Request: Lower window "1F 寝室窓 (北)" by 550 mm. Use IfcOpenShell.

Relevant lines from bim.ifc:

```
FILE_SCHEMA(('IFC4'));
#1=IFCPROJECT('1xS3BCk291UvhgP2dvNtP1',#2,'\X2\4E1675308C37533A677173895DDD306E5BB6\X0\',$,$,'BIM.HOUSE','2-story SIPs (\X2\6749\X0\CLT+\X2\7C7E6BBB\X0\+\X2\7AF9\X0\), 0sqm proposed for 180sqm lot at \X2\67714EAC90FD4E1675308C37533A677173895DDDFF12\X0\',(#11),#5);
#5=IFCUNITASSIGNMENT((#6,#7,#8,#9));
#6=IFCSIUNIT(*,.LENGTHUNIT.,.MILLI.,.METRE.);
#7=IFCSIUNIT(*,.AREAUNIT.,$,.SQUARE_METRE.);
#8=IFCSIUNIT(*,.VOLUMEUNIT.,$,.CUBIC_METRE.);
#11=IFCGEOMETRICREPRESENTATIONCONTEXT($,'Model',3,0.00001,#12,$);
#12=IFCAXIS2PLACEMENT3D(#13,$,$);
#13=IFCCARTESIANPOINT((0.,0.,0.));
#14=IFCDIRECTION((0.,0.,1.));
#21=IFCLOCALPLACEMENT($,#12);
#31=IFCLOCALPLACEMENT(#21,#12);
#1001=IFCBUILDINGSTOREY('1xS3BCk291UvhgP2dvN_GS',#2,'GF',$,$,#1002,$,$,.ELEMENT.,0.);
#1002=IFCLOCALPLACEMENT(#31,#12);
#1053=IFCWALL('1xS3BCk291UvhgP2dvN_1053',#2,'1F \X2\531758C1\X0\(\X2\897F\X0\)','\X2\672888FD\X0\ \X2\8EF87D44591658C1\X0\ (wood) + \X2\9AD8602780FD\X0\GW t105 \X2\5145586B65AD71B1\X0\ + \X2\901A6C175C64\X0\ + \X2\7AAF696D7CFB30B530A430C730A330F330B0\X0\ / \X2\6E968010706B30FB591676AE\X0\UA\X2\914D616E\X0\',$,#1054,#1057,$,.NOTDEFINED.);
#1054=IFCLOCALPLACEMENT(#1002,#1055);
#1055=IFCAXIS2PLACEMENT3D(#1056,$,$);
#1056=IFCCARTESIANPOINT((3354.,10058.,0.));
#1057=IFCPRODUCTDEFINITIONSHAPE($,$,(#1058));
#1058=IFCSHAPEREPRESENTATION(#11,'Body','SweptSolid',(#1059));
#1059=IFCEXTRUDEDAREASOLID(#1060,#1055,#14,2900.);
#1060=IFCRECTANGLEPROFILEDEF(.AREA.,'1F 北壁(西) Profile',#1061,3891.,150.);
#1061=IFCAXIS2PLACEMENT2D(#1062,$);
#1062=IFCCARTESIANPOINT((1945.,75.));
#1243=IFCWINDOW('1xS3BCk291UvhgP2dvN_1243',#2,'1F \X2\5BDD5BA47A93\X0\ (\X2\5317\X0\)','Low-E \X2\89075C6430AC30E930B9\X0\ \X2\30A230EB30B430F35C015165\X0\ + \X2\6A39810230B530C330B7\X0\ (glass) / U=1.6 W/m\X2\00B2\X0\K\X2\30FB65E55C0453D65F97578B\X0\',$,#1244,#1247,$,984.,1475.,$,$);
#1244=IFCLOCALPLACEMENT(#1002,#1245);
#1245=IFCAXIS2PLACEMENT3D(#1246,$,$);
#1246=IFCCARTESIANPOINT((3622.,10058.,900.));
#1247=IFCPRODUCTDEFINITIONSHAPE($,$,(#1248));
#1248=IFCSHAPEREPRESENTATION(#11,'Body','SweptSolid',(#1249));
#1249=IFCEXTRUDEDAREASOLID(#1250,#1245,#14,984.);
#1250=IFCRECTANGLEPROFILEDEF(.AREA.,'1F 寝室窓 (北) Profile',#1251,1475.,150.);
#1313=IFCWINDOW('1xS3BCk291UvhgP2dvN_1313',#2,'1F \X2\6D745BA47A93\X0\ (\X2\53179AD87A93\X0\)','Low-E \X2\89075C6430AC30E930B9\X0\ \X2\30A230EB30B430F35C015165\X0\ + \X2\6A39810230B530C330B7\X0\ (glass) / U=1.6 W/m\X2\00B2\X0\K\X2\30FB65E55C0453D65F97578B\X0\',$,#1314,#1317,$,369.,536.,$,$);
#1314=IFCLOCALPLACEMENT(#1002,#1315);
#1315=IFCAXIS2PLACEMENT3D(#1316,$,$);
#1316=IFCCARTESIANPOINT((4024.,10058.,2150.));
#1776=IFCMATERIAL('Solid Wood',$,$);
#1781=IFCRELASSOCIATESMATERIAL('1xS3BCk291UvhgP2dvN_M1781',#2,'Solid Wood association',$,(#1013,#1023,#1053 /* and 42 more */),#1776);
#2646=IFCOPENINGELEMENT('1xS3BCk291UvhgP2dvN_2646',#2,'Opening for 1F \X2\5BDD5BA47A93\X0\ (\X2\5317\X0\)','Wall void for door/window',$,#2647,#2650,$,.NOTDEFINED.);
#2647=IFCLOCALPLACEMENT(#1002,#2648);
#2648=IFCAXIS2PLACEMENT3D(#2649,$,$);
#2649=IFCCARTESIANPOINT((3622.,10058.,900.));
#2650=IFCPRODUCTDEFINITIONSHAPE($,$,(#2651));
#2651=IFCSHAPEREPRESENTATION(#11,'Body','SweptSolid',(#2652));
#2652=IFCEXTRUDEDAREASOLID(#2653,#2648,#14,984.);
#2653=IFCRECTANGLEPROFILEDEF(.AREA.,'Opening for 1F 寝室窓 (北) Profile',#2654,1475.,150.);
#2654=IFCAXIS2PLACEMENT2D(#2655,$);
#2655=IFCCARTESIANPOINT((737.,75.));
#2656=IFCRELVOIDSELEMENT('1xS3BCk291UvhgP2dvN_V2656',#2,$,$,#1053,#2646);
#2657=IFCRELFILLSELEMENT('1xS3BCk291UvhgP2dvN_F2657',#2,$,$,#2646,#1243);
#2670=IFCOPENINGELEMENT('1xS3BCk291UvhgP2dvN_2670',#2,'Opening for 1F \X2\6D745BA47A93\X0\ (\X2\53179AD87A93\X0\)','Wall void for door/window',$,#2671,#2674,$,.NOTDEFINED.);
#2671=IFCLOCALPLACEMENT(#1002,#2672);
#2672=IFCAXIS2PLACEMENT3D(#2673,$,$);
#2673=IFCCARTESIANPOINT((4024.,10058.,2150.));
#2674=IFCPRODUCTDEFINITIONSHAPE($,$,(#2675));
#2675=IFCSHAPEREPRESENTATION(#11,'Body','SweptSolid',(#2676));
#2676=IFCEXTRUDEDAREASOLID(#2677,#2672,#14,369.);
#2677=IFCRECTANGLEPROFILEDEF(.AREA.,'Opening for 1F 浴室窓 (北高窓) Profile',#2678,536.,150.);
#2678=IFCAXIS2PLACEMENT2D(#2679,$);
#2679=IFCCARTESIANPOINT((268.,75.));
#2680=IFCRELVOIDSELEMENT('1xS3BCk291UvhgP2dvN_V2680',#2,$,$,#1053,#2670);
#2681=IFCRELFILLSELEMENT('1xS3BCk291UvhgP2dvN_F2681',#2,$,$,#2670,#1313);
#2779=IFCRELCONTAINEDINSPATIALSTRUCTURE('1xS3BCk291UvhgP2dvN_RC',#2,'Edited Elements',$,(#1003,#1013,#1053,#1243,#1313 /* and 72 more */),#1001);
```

```python
import numpy as np
import ifcopenshell
import ifcopenshell.api.geometry
import ifcopenshell.util.placement
import ifcopenshell.util.unit

model = ifcopenshell.open("bim.ifc")
unit_scale = ifcopenshell.util.unit.calculate_unit_scale(model)

window = model.by_guid("1xS3BCk291UvhgP2dvN_1243")
opening = window.FillsVoids[0].RelatingOpeningElement
dz = -550.0

shift = np.array([0.0, 0.0, dz])
# The window is not placed relative to its opening, so move both.
for product in (opening, window):
    matrix = ifcopenshell.util.placement.get_local_placement(product.ObjectPlacement)
    matrix[:3, 3] += shift
    ifcopenshell.api.geometry.edit_object_placement(model, product=product, matrix=matrix, is_si=False)

print(f"moved by {dz * unit_scale:+.3f} m")

model.write("bim-out.ifc")
```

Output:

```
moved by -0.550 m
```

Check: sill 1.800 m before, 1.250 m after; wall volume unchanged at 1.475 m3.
